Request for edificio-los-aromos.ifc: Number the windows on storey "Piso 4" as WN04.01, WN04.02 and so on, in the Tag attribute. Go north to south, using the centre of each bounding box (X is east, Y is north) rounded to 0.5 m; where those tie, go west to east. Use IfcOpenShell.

First a look at what the model holds.

```python
import ifcopenshell
import ifcopenshell.util.element
import ifcopenshell.util.placement

model = ifcopenshell.open("edificio-los-aromos.ifc")
print(model.schema)
storey = next(s for s in model.by_type("IfcBuildingStorey") if s.Name == "Piso 4")
windows = [e for e in ifcopenshell.util.element.get_decomposition(storey) if e.is_a("IfcWindow")]
for e in sorted(windows, key=lambda e: e.id()):
    origin = ifcopenshell.util.placement.get_local_placement(e.ObjectPlacement)[:3, 3]
    print(e.id(), e.Tag, e.Name, origin.round(2) + 0.0, sep=" | ")
```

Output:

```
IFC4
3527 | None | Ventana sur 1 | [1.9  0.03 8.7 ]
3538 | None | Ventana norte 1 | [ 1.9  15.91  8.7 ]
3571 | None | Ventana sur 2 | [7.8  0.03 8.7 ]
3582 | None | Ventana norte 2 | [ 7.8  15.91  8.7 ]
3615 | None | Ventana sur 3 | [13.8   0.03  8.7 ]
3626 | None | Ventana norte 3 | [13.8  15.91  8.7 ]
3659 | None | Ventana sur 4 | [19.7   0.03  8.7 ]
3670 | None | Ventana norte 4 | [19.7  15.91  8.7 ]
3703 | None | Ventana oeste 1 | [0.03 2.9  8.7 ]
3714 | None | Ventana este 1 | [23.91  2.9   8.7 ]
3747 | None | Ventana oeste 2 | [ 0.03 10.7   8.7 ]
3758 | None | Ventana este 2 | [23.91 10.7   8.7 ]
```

```python
import ifcopenshell
import ifcopenshell.geom
import ifcopenshell.util.element
import ifcopenshell.util.shape

model = ifcopenshell.open("edificio-los-aromos.ifc")
settings = ifcopenshell.geom.settings()
settings.set("use-world-coords", True)


def centre(element):
    shape = ifcopenshell.geom.create_shape(settings, element)
    return ifcopenshell.util.shape.get_bbox_centroid(shape.geometry)


storey = next(s for s in model.by_type("IfcBuildingStorey") if s.Name == "Piso 4")
windows = [e for e in ifcopenshell.util.element.get_decomposition(storey) if e.is_a("IfcWindow")]

# Insertion points can sit at a corner or the storey origin, so sort by the geometry (in metres).
centres = {e: centre(e) for e in windows}
windows.sort(key=lambda e: (-round(centres[e][1] / 0.5), centres[e][0]))

for i, e in enumerate(windows, start=1):
    number = f"WN04.{i:02d}"
    e.Tag = number
    print(e.id(), number)

model.write("edificio-los-aromos-out.ifc")
```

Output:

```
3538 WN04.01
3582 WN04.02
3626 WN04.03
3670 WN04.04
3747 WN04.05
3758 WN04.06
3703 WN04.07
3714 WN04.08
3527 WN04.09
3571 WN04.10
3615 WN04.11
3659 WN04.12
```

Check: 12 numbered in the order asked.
